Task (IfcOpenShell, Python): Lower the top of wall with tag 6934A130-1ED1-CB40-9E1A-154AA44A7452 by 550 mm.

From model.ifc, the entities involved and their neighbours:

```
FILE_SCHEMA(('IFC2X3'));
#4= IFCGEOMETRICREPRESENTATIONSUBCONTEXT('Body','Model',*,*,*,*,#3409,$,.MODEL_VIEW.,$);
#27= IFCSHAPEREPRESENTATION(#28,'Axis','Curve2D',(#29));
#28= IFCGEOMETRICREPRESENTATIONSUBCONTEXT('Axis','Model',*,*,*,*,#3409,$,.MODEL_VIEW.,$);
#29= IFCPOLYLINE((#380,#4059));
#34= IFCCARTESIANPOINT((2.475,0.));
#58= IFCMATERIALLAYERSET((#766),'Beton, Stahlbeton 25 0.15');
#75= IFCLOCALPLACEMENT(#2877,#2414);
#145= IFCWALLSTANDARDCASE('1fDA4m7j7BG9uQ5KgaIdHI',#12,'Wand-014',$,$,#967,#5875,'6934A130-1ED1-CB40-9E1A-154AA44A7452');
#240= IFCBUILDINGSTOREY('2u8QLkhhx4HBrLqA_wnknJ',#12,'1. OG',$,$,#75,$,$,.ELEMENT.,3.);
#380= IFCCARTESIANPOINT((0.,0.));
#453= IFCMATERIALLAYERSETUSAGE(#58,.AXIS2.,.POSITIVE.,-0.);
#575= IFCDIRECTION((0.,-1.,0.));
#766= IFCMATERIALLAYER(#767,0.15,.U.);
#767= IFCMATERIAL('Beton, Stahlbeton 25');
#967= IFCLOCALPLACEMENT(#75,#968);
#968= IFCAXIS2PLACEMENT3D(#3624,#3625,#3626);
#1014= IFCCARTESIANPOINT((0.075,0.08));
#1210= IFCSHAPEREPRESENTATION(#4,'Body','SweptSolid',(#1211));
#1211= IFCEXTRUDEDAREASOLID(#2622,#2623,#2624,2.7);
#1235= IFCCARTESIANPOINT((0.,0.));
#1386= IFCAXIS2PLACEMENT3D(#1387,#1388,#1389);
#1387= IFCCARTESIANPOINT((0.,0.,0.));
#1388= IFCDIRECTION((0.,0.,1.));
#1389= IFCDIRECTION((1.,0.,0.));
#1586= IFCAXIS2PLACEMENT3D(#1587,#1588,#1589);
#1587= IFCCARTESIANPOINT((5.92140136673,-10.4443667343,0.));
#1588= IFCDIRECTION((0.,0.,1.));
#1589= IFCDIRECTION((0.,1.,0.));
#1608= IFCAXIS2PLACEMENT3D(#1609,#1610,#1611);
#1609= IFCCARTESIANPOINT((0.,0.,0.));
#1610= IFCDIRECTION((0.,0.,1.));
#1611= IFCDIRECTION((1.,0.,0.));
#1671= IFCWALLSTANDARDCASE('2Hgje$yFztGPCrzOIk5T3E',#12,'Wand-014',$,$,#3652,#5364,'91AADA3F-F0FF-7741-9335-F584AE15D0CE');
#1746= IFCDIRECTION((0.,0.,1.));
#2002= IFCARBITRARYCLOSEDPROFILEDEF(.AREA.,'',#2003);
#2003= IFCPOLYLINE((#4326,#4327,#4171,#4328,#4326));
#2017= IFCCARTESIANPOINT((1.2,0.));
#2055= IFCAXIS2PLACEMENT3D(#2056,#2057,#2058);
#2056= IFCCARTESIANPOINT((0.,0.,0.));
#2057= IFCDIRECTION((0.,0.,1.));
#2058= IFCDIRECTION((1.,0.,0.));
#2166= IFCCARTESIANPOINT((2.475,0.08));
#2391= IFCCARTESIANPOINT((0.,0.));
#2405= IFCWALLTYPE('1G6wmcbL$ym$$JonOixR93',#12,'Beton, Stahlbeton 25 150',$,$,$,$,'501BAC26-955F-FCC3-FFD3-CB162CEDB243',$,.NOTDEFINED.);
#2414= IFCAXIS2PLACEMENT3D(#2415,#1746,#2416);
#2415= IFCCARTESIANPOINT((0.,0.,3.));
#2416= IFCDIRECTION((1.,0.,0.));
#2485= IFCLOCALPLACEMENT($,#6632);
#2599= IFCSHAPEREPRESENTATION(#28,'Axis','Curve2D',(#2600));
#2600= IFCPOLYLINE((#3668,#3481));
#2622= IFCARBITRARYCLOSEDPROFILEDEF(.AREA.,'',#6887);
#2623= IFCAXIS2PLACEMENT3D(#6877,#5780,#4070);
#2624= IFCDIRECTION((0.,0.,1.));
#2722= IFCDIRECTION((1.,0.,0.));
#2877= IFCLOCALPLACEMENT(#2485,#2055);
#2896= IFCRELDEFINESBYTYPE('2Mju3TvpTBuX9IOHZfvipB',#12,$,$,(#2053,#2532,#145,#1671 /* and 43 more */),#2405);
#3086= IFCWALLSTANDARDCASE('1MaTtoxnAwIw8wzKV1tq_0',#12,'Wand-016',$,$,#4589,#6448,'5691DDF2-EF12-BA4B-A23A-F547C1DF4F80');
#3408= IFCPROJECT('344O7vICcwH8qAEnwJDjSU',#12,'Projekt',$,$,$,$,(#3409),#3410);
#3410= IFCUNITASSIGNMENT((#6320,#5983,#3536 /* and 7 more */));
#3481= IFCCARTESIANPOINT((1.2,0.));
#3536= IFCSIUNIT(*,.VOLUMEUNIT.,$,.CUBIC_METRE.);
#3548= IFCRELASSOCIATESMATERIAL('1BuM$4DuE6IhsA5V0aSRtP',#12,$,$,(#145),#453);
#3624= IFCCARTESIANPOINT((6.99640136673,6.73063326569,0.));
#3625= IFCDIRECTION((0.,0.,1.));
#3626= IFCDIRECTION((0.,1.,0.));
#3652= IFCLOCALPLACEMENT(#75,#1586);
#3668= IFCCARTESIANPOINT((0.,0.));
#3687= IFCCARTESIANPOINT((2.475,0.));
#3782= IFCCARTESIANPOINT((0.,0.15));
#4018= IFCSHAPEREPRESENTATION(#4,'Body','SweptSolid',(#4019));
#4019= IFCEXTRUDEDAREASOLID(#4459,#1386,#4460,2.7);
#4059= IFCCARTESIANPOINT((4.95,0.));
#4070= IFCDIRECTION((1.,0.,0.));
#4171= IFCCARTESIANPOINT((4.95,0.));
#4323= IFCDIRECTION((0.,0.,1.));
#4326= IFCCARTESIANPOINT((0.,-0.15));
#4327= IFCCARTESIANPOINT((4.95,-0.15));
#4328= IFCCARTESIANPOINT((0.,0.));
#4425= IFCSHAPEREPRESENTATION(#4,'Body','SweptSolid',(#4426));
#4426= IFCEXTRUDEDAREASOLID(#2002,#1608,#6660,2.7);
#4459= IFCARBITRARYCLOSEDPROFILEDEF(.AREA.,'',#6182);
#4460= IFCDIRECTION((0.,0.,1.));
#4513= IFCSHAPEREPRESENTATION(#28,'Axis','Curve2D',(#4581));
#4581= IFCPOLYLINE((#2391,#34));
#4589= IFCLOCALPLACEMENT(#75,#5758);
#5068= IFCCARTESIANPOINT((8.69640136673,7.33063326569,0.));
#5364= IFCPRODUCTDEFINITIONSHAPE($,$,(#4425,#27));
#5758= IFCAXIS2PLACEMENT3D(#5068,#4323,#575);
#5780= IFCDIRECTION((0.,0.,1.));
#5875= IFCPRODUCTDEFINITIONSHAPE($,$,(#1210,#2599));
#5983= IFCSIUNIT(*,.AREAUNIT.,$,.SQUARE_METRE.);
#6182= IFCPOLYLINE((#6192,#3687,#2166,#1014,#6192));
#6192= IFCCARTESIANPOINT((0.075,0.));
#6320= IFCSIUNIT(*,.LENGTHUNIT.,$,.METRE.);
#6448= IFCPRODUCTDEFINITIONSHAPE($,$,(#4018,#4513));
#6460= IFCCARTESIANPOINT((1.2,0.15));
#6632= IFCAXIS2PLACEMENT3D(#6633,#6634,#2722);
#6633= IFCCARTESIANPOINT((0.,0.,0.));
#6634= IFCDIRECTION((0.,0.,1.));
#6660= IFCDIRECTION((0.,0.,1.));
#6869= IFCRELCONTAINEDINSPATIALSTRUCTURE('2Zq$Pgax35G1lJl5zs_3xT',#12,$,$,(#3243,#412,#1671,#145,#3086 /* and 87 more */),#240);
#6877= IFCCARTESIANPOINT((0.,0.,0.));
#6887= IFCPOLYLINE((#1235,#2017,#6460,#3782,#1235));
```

```python
import ifcopenshell
import ifcopenshell.geom
import ifcopenshell.util.representation
import ifcopenshell.util.shape
import ifcopenshell.util.unit

model = ifcopenshell.open("model.ifc")
unit_scale = ifcopenshell.util.unit.calculate_unit_scale(model)
settings = ifcopenshell.geom.settings()


def volume(element):
    """Net volume in cubic metres, openings subtracted."""
    shape = ifcopenshell.geom.create_shape(settings, element)
    return ifcopenshell.util.shape.get_volume(shape.geometry)


wall = model.by_guid("1fDA4m7j7BG9uQ5KgaIdHI")
before = volume(wall)

body = ifcopenshell.util.representation.get_representation(wall, "Model", "Body")
solid = body.Items[0]
old_height = solid.Depth
solid.Depth -= 0.55 / unit_scale
after = volume(wall)

print(f"height {old_height:g} -> {solid.Depth:g}, volume {before:.3f} -> {after:.3f} m3")

model.write("model-out.ifc")
```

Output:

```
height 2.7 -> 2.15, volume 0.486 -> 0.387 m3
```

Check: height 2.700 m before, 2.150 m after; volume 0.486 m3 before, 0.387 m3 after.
